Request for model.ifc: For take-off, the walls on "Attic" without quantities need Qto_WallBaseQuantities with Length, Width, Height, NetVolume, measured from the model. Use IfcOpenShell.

First a look at what the model holds.

```python
import ifcopenshell
import ifcopenshell.util.element
import ifcopenshell.util.unit

model = ifcopenshell.open("model.ifc")
print(model.schema)
for unit_type in ("LENGTHUNIT", "AREAUNIT", "VOLUMEUNIT"):
    print(unit_type, ifcopenshell.util.unit.calculate_unit_scale(model, unit_type))
storey = next(s for s in model.by_type("IfcBuildingStorey") if s.Name == "Attic")
walls = [e for e in ifcopenshell.util.element.get_decomposition(storey) if e.is_a("IfcWall")]
for e in sorted(walls, key=lambda e: e.id()):
    print(e.id(), e.is_a(), e.Name, list(ifcopenshell.util.element.get_psets(e, qtos_only=True)), sep=" | ")
```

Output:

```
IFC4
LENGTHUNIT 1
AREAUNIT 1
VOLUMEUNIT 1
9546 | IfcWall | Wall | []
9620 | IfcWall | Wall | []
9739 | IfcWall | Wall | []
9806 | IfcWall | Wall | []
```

```python
import ifcopenshell
import ifcopenshell.api.pset
import ifcopenshell.geom
import ifcopenshell.util.element
import ifcopenshell.util.shape
import ifcopenshell.util.unit

model = ifcopenshell.open("model.ifc")
unit_scale = ifcopenshell.util.unit.calculate_unit_scale(model)
volume_scale = ifcopenshell.util.unit.calculate_unit_scale(model, "VOLUMEUNIT")
settings = ifcopenshell.geom.settings()

storey = next(s for s in model.by_type("IfcBuildingStorey") if s.Name == "Attic")
walls = [e for e in ifcopenshell.util.element.get_decomposition(storey) if e.is_a("IfcWall")]

for e in sorted(walls, key=lambda e: e.id()):
    if ifcopenshell.util.element.get_psets(e, qtos_only=True, should_inherit=False):
        continue
    # Geometry comes back in metres, in the element's own axes.
    shape = ifcopenshell.geom.create_shape(settings, e)
    values = {
        "Length": ifcopenshell.util.shape.get_x(shape.geometry) / unit_scale,
        "Width": ifcopenshell.util.shape.get_y(shape.geometry) / unit_scale,
        "Height": ifcopenshell.util.shape.get_z(shape.geometry) / unit_scale,
        "NetVolume": ifcopenshell.util.shape.get_volume(shape.geometry) / volume_scale,
    }
    qto = ifcopenshell.api.pset.add_qto(model, product=e, name="Qto_WallBaseQuantities")
    ifcopenshell.api.pset.edit_qto(model, qto=qto, properties=values)
    print(e.id(), {k: round(v, 3) for k, v in values.items()})

model.write("model_updated.ifc")
```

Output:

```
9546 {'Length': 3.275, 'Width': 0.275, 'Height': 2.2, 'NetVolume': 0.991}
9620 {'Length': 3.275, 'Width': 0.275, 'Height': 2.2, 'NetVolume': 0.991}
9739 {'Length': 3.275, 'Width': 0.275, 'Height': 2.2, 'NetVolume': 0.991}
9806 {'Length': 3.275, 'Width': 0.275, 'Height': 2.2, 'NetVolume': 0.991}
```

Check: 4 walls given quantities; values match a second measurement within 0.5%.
